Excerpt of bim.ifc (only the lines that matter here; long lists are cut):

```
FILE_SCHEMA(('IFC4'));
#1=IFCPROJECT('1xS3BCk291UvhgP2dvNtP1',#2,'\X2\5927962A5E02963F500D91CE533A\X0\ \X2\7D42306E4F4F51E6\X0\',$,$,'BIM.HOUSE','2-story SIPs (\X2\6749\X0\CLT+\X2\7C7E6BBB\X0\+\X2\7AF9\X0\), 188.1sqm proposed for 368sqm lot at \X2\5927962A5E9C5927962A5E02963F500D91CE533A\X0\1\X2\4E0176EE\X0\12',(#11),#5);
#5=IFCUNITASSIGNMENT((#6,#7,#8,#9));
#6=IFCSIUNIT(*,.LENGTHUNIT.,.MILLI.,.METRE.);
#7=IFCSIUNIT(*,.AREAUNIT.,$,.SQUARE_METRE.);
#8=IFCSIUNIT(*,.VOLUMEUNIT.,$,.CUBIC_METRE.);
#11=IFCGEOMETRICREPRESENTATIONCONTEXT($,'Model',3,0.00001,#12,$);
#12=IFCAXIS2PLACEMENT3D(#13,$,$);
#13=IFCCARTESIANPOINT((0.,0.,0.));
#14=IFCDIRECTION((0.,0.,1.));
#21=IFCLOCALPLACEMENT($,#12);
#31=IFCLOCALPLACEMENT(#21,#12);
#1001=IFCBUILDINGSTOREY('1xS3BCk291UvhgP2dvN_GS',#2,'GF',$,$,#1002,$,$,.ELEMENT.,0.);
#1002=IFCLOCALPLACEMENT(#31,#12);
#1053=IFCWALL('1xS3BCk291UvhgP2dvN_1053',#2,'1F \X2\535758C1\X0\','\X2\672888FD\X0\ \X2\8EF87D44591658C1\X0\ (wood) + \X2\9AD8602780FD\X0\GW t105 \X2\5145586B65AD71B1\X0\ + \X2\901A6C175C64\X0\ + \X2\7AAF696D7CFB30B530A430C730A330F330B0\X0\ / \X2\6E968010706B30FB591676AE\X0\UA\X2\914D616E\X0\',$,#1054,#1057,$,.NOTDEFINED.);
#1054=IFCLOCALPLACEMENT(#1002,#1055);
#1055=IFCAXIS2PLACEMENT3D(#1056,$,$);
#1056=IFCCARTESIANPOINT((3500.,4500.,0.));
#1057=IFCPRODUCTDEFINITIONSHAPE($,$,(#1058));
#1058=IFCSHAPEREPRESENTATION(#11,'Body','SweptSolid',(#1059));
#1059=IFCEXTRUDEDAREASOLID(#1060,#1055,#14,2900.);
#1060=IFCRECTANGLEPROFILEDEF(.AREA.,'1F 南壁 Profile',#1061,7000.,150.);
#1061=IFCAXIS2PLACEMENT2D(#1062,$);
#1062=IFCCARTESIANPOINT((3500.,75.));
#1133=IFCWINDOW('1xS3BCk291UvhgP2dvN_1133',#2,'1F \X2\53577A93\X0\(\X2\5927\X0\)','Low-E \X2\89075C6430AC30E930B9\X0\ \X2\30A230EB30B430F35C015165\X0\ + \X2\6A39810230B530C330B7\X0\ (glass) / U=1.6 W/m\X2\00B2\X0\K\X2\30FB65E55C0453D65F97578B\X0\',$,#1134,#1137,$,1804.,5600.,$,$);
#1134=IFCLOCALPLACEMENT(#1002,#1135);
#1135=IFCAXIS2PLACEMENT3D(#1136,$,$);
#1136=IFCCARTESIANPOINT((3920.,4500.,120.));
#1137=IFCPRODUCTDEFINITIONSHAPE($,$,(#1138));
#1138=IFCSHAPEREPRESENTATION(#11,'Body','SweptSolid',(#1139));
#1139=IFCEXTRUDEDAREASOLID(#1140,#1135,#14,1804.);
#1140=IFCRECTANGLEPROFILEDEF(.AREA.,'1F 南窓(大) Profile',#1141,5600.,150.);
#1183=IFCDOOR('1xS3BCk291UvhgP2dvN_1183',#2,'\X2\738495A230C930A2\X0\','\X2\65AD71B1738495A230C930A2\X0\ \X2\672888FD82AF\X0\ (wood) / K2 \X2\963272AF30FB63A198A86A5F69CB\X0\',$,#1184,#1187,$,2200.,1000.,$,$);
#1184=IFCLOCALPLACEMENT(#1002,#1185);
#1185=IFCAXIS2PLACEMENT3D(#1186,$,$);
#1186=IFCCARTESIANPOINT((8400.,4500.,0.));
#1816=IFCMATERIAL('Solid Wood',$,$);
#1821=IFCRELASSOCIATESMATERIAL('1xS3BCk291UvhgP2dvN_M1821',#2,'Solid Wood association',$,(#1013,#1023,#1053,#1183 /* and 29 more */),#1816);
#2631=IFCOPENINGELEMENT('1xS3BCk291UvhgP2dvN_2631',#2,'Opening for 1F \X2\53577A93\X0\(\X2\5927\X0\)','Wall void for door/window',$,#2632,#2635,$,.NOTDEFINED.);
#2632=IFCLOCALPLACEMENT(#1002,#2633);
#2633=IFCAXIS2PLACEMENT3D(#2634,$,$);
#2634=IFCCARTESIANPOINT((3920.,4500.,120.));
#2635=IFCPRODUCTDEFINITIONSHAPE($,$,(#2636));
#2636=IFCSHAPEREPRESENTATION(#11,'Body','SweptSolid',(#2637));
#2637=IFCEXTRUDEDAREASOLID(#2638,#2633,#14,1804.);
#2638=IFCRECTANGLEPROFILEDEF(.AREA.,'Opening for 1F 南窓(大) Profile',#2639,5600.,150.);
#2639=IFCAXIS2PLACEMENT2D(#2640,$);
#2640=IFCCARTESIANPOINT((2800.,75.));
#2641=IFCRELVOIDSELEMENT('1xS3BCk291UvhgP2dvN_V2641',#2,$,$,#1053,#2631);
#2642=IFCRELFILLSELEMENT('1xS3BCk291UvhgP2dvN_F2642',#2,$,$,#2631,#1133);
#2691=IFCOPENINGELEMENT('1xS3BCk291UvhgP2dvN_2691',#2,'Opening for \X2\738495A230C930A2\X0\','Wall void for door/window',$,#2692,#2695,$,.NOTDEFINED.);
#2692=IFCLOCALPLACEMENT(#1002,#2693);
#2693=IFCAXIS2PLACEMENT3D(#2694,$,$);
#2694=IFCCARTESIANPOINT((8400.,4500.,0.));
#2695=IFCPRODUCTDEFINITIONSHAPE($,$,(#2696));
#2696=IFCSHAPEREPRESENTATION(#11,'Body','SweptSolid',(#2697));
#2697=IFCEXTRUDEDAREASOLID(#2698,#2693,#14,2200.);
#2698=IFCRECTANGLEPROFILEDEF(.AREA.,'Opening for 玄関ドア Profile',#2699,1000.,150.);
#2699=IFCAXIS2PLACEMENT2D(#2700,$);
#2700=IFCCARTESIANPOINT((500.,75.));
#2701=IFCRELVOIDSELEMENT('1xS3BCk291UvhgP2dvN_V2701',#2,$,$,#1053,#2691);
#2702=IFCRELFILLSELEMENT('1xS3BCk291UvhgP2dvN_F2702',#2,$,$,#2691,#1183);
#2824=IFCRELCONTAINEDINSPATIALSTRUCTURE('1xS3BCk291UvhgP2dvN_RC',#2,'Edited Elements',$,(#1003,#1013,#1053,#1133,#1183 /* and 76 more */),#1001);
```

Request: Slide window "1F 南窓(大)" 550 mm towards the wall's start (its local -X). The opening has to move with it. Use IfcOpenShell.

```python
import ifcopenshell
import ifcopenshell.api.geometry
import ifcopenshell.util.placement

model = ifcopenshell.open("bim.ifc")

window = model.by_guid("1xS3BCk291UvhgP2dvN_1133")
opening = window.FillsVoids[0].RelatingOpeningElement
wall = opening.VoidsElements[0].RelatingBuildingElement

wall_matrix = ifcopenshell.util.placement.get_local_placement(wall.ObjectPlacement)
shift = wall_matrix[:3, 0] * -550.0
before = ifcopenshell.util.placement.get_local_placement(window.ObjectPlacement)[:3, 3].copy()

# The window is not placed relative to its opening, so move both.
for product in (opening, window):
    matrix = ifcopenshell.util.placement.get_local_placement(product.ObjectPlacement)
    matrix[:3, 3] += shift
    ifcopenshell.api.geometry.edit_object_placement(model, product=product, matrix=matrix, is_si=False)

after = ifcopenshell.util.placement.get_local_placement(window.ObjectPlacement)[:3, 3]
print("window moved by", (after - before).round(3) + 0.0)

model.write("bim_rev.ifc")
```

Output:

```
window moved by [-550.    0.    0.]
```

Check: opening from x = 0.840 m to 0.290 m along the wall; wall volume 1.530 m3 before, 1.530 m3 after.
